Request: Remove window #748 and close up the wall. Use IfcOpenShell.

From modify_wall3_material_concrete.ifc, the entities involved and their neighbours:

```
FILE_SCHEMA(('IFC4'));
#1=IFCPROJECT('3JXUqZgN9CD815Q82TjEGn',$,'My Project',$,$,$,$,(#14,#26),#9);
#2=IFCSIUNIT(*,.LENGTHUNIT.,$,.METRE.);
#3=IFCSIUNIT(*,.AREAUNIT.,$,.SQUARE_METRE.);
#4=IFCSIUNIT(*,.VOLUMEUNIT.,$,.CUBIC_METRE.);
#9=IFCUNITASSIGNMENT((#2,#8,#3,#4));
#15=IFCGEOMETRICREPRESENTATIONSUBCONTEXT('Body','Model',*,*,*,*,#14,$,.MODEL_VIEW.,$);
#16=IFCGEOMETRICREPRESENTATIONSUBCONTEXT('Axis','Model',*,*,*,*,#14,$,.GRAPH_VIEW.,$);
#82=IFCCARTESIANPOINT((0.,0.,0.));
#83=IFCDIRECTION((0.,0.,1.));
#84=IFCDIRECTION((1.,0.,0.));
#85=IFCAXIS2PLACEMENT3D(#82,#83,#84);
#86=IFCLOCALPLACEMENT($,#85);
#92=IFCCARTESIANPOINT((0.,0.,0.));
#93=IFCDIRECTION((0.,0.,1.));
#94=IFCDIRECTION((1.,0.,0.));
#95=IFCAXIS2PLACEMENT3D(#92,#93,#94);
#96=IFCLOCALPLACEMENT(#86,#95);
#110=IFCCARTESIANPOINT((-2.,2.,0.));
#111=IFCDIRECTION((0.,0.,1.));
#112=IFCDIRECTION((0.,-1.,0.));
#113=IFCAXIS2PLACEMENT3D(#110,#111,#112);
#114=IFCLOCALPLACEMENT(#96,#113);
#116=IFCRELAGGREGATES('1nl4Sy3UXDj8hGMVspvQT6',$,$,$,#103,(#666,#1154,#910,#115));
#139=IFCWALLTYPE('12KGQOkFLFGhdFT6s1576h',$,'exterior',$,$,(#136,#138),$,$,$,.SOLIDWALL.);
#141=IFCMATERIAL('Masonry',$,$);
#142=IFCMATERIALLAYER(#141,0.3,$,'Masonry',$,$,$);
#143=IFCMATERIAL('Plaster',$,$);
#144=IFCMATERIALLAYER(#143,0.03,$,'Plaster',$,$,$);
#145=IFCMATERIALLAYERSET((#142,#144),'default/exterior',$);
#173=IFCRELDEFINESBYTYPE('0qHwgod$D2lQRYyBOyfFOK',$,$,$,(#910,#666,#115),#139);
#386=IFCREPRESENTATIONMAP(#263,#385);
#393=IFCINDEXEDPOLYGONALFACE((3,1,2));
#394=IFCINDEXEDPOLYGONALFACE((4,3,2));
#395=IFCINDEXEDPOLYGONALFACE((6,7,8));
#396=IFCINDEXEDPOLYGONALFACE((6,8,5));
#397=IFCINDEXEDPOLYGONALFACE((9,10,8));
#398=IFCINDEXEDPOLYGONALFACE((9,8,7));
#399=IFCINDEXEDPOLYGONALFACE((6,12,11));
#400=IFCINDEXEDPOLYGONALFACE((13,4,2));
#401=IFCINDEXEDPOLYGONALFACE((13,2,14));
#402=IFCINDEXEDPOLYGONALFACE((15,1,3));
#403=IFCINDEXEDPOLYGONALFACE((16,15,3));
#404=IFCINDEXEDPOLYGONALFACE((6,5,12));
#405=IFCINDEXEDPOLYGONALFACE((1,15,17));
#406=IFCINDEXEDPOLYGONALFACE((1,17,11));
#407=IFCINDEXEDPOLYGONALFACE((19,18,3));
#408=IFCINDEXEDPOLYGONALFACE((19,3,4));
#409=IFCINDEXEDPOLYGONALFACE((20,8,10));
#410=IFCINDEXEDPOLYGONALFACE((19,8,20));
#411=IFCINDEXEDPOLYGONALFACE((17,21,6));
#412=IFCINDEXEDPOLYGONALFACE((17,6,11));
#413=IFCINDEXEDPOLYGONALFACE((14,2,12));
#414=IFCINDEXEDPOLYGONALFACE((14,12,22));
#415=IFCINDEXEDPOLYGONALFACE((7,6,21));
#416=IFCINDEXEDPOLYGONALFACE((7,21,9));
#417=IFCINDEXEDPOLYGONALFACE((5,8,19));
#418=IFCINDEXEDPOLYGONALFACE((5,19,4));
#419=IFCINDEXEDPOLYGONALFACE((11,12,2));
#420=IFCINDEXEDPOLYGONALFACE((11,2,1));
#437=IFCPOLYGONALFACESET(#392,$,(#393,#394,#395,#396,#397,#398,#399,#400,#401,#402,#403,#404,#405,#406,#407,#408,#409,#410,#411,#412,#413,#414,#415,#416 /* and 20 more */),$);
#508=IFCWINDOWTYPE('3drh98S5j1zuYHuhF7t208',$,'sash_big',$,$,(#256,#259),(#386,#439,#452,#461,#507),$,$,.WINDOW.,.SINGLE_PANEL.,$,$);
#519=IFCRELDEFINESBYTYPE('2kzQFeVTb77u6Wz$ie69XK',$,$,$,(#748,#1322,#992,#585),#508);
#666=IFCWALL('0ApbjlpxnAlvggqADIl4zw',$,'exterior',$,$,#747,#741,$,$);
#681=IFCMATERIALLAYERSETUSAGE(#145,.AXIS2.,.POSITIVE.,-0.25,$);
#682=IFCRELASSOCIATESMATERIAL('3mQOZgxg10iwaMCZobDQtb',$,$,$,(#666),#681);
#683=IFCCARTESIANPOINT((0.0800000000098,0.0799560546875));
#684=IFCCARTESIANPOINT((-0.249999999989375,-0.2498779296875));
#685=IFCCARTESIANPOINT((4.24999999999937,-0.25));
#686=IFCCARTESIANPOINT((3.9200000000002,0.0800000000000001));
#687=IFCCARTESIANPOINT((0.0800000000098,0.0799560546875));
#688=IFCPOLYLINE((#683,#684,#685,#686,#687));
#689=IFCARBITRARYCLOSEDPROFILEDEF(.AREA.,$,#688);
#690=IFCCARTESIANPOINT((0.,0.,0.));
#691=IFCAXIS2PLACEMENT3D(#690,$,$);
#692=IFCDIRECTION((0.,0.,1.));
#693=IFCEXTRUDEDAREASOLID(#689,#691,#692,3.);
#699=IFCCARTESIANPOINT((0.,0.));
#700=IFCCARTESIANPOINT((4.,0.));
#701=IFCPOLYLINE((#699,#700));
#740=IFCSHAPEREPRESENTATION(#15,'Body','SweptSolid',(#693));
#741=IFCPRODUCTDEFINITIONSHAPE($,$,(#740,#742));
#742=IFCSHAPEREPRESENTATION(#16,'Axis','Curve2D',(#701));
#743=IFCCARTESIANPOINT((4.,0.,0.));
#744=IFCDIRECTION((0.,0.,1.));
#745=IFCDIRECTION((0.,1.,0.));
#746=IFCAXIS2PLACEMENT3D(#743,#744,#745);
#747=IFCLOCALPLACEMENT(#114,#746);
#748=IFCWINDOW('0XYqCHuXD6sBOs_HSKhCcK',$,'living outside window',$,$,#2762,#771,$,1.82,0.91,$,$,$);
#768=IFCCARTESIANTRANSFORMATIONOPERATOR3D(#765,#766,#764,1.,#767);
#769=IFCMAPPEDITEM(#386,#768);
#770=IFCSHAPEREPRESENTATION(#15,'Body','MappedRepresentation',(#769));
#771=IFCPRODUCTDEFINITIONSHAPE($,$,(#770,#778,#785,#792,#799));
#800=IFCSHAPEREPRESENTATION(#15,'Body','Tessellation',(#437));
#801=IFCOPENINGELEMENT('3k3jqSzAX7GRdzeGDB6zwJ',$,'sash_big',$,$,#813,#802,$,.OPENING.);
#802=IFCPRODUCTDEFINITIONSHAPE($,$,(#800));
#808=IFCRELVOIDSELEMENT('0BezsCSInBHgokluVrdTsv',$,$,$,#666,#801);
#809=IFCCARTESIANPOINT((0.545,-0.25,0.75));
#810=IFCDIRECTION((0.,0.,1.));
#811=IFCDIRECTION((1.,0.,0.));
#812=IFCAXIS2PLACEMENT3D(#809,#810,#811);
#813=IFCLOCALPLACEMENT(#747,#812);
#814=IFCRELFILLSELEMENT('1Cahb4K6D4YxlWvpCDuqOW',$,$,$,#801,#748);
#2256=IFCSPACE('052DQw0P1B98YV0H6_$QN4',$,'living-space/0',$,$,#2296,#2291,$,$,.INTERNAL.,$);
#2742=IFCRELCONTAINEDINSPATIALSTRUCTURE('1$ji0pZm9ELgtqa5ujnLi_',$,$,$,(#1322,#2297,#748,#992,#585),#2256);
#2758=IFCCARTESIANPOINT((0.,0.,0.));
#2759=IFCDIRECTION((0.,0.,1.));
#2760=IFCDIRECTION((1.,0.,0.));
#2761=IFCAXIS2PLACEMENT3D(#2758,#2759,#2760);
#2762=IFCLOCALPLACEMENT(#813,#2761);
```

```python
import ifcopenshell
import ifcopenshell.api.feature
import ifcopenshell.api.root
import ifcopenshell.geom
import ifcopenshell.util.shape

model = ifcopenshell.open("modify_wall3_material_concrete.ifc")
settings = ifcopenshell.geom.settings()


def volume(element):
    """Net volume in cubic metres, openings subtracted."""
    shape = ifcopenshell.geom.create_shape(settings, element)
    return ifcopenshell.util.shape.get_volume(shape.geometry)


window = model.by_guid("0XYqCHuXD6sBOs_HSKhCcK")
opening = window.FillsVoids[0].RelatingOpeningElement
wall = opening.VoidsElements[0].RelatingBuildingElement
before = volume(wall)

ifcopenshell.api.root.remove_product(model, product=window)
ifcopenshell.api.feature.remove_feature(model, feature=opening)

after = volume(wall)

print(f"wall volume {before:.3f} -> {after:.3f} m3")

model.write("modify_wall3_material_concrete-out.ifc")
```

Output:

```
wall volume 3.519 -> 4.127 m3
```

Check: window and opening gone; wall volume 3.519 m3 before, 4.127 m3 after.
